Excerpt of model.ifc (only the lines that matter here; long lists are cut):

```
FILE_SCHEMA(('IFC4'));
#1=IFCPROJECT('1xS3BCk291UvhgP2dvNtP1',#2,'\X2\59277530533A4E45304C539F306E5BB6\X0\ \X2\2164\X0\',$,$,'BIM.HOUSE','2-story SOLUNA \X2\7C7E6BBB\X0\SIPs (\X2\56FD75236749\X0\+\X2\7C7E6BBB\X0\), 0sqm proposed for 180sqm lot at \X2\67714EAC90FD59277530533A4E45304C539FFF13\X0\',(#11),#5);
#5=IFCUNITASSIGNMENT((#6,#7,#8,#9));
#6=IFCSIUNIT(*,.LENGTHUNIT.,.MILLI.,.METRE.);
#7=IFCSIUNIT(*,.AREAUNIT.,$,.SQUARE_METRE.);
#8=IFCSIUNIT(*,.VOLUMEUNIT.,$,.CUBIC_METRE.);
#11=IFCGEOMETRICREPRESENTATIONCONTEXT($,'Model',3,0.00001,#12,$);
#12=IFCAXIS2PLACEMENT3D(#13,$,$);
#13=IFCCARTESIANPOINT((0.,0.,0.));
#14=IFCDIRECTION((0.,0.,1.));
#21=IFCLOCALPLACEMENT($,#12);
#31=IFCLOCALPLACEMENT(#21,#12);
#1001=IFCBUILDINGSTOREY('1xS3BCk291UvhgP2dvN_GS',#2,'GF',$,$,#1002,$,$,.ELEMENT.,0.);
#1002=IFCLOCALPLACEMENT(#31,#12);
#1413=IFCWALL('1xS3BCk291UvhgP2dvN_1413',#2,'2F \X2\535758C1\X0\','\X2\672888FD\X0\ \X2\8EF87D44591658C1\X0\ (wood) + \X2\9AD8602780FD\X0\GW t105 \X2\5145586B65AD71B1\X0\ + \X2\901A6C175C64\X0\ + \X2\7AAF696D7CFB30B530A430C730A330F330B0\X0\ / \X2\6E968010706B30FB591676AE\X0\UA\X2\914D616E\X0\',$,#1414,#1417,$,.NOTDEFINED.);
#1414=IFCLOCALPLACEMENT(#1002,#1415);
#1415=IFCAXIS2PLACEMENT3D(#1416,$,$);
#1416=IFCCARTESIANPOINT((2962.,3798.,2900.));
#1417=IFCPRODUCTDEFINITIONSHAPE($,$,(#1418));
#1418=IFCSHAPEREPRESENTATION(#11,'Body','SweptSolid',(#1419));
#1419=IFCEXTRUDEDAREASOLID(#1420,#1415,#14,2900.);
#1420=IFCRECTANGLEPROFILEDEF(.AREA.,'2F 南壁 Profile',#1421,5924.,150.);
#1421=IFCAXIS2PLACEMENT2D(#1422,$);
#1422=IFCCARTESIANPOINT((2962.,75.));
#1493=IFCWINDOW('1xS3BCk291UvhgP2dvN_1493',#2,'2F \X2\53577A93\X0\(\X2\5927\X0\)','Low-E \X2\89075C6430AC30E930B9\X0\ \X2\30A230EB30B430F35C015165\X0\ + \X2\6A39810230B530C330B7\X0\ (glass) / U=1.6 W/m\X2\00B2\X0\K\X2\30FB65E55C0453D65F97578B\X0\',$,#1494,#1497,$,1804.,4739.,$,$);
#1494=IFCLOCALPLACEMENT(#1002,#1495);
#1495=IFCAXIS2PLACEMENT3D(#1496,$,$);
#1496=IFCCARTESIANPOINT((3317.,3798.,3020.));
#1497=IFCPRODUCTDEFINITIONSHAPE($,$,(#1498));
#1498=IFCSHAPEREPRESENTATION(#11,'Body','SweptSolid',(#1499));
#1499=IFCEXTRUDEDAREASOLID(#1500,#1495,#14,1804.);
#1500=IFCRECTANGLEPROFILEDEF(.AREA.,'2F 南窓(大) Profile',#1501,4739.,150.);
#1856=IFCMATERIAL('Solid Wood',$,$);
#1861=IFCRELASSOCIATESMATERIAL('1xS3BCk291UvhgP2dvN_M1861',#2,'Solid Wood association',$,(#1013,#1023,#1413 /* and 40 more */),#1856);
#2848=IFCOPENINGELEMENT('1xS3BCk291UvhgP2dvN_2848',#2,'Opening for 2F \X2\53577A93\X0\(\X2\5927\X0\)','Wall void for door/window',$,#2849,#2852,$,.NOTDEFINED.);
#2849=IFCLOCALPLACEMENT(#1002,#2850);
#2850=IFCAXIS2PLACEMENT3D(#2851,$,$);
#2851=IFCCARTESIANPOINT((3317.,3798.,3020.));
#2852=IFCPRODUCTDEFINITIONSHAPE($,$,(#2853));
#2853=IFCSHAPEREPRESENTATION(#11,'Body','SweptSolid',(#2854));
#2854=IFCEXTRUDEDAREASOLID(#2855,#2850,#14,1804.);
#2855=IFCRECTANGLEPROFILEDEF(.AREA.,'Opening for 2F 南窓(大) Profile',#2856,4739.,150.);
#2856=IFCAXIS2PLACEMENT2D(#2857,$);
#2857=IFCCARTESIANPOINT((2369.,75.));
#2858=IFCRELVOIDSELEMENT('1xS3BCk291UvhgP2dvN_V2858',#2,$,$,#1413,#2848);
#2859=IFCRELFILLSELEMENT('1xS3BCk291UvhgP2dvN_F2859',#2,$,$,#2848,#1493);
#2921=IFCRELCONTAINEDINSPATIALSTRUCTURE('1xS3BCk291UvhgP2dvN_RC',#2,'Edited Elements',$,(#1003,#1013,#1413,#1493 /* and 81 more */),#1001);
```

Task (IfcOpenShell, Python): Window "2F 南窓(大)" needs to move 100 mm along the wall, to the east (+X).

```python
import ifcopenshell
import ifcopenshell.api.geometry
import ifcopenshell.util.placement

model = ifcopenshell.open("model.ifc")

window = model.by_guid("1xS3BCk291UvhgP2dvN_1493")
opening = window.FillsVoids[0].RelatingOpeningElement
wall = opening.VoidsElements[0].RelatingBuildingElement

wall_matrix = ifcopenshell.util.placement.get_local_placement(wall.ObjectPlacement)
shift = wall_matrix[:3, 0] * 100.0
before = ifcopenshell.util.placement.get_local_placement(window.ObjectPlacement)[:3, 3].copy()

# The window is not placed relative to its opening, so move both.
for product in (opening, window):
    matrix = ifcopenshell.util.placement.get_local_placement(product.ObjectPlacement)
    matrix[:3, 3] += shift
    ifcopenshell.api.geometry.edit_object_placement(model, product=product, matrix=matrix, is_si=False)

after = ifcopenshell.util.placement.get_local_placement(window.ObjectPlacement)[:3, 3]
print("window moved by", (after - before).round(3) + 0.0)

model.write("model_rev.ifc")
```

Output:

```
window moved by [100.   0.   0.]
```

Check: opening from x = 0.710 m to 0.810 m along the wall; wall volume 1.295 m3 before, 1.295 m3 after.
